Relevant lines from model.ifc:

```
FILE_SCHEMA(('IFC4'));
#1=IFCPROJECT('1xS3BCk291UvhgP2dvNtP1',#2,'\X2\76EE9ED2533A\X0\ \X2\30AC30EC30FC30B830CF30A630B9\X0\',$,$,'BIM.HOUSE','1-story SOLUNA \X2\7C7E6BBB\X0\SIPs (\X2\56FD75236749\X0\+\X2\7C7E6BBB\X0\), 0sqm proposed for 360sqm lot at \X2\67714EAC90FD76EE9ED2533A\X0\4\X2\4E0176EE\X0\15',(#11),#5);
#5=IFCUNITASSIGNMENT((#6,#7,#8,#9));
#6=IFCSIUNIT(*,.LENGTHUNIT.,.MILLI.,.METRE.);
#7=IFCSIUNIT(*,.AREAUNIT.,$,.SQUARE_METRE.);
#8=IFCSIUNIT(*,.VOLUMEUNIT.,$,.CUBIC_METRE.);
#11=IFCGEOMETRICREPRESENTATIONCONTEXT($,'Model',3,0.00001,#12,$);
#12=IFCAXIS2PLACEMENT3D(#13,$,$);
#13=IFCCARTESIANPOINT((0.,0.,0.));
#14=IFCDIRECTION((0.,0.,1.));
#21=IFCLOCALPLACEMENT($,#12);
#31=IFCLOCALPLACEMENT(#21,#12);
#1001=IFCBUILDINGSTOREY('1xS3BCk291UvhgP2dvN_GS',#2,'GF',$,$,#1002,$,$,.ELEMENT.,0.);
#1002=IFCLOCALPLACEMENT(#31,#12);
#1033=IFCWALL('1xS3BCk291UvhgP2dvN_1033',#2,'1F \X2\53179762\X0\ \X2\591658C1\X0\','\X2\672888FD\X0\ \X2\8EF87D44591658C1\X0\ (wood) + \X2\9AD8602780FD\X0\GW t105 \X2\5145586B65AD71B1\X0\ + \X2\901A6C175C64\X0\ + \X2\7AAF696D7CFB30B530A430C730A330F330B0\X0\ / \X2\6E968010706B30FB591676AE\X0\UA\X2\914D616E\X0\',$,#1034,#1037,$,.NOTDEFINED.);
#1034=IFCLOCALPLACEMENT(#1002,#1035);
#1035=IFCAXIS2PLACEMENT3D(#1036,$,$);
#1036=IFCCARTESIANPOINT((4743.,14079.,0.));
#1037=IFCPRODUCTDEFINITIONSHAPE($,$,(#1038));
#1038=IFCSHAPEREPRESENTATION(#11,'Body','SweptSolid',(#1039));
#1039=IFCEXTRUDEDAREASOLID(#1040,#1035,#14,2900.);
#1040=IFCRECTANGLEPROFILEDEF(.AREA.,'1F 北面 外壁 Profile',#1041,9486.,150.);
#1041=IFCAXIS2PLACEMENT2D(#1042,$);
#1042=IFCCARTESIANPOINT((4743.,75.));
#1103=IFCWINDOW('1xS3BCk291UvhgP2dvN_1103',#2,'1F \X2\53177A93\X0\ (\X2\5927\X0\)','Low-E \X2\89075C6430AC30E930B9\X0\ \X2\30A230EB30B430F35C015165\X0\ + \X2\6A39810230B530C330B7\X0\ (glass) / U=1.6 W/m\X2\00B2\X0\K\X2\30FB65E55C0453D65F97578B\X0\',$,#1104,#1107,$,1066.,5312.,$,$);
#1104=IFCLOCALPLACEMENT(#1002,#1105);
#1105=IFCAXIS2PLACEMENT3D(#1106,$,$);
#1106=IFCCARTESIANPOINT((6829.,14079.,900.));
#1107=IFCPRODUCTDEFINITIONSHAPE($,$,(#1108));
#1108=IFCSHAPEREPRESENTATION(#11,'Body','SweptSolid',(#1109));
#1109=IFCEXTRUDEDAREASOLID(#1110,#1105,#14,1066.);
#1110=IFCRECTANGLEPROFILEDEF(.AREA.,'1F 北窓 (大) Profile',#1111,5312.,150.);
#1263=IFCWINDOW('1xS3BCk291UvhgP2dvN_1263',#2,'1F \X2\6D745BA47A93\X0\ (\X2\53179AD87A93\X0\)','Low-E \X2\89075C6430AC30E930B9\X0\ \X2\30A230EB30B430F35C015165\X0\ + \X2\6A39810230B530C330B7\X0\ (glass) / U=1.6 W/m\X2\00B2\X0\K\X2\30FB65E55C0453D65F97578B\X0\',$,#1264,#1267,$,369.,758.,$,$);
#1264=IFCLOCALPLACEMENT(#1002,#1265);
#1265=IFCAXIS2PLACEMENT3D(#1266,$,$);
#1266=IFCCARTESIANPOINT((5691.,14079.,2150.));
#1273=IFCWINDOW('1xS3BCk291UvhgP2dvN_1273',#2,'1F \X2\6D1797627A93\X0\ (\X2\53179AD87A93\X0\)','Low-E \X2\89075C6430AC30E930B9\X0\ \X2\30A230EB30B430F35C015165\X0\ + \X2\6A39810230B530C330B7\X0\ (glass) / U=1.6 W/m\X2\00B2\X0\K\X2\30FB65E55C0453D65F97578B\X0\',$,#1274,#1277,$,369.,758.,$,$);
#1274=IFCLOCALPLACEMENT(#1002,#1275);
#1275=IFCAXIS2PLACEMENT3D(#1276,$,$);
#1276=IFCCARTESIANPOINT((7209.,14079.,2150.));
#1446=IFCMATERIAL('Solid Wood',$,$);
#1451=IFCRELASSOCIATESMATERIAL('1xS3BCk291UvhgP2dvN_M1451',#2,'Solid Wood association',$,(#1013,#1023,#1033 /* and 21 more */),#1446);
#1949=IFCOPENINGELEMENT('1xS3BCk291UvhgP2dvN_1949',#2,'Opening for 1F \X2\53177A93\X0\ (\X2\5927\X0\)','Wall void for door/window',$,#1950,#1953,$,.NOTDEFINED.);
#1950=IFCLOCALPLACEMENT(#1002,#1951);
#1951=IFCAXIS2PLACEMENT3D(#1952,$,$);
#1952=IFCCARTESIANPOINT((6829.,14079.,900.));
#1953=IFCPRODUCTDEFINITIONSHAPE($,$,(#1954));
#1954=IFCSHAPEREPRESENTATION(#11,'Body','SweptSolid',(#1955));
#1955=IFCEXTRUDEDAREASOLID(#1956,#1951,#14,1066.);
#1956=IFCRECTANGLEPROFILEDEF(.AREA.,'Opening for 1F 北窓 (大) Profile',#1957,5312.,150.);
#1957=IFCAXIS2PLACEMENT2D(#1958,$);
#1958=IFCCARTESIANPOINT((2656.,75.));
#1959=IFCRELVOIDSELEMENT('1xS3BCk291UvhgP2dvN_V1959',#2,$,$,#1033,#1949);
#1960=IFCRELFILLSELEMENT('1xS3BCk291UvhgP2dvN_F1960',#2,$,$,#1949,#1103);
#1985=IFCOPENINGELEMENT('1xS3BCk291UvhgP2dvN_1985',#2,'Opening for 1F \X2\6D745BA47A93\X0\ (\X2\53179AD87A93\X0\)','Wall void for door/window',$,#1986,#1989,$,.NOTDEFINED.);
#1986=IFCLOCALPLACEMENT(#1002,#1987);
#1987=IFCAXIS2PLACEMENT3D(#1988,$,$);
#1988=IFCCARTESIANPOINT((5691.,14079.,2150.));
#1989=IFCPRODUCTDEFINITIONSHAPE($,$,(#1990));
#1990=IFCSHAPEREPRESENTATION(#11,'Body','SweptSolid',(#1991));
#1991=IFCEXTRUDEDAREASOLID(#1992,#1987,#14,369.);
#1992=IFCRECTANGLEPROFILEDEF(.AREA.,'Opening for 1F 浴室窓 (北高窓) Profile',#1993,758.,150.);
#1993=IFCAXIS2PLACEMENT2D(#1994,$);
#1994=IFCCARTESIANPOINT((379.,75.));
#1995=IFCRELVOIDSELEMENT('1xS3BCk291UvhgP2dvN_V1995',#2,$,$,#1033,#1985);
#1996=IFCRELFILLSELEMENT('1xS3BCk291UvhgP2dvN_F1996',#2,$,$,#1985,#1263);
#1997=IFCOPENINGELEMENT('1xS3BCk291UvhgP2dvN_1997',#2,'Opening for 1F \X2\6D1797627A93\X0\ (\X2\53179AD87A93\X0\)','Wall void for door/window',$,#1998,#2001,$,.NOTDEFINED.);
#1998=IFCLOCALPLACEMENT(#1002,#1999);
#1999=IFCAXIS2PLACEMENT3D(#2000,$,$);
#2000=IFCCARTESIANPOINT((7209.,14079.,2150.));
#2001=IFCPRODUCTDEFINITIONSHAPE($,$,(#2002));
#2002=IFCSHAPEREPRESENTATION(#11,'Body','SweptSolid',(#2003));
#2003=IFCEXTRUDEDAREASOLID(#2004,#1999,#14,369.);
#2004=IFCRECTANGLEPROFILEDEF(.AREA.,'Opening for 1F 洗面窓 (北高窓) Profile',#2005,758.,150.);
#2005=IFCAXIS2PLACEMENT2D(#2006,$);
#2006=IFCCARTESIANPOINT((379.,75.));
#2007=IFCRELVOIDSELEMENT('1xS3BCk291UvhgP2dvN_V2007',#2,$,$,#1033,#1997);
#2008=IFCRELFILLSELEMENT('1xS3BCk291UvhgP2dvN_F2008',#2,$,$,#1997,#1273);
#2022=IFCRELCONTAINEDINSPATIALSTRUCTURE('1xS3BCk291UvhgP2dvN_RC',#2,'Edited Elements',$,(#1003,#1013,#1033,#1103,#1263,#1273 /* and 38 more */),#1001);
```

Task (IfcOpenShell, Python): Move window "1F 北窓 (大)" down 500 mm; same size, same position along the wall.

```python
import numpy as np
import ifcopenshell
import ifcopenshell.api.geometry
import ifcopenshell.util.placement
import ifcopenshell.util.unit

model = ifcopenshell.open("model.ifc")
unit_scale = ifcopenshell.util.unit.calculate_unit_scale(model)

window = model.by_guid("1xS3BCk291UvhgP2dvN_1103")
opening = window.FillsVoids[0].RelatingOpeningElement
dz = -0.5 / unit_scale

shift = np.array([0.0, 0.0, dz])
# The window is not placed relative to its opening, so move both.
for product in (opening, window):
    matrix = ifcopenshell.util.placement.get_local_placement(product.ObjectPlacement)
    matrix[:3, 3] += shift
    ifcopenshell.api.geometry.edit_object_placement(model, product=product, matrix=matrix, is_si=False)

print(f"moved by {dz * unit_scale:+.3f} m")

model.write("model_edited.ifc")
```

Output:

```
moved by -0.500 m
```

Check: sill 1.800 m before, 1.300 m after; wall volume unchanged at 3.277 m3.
